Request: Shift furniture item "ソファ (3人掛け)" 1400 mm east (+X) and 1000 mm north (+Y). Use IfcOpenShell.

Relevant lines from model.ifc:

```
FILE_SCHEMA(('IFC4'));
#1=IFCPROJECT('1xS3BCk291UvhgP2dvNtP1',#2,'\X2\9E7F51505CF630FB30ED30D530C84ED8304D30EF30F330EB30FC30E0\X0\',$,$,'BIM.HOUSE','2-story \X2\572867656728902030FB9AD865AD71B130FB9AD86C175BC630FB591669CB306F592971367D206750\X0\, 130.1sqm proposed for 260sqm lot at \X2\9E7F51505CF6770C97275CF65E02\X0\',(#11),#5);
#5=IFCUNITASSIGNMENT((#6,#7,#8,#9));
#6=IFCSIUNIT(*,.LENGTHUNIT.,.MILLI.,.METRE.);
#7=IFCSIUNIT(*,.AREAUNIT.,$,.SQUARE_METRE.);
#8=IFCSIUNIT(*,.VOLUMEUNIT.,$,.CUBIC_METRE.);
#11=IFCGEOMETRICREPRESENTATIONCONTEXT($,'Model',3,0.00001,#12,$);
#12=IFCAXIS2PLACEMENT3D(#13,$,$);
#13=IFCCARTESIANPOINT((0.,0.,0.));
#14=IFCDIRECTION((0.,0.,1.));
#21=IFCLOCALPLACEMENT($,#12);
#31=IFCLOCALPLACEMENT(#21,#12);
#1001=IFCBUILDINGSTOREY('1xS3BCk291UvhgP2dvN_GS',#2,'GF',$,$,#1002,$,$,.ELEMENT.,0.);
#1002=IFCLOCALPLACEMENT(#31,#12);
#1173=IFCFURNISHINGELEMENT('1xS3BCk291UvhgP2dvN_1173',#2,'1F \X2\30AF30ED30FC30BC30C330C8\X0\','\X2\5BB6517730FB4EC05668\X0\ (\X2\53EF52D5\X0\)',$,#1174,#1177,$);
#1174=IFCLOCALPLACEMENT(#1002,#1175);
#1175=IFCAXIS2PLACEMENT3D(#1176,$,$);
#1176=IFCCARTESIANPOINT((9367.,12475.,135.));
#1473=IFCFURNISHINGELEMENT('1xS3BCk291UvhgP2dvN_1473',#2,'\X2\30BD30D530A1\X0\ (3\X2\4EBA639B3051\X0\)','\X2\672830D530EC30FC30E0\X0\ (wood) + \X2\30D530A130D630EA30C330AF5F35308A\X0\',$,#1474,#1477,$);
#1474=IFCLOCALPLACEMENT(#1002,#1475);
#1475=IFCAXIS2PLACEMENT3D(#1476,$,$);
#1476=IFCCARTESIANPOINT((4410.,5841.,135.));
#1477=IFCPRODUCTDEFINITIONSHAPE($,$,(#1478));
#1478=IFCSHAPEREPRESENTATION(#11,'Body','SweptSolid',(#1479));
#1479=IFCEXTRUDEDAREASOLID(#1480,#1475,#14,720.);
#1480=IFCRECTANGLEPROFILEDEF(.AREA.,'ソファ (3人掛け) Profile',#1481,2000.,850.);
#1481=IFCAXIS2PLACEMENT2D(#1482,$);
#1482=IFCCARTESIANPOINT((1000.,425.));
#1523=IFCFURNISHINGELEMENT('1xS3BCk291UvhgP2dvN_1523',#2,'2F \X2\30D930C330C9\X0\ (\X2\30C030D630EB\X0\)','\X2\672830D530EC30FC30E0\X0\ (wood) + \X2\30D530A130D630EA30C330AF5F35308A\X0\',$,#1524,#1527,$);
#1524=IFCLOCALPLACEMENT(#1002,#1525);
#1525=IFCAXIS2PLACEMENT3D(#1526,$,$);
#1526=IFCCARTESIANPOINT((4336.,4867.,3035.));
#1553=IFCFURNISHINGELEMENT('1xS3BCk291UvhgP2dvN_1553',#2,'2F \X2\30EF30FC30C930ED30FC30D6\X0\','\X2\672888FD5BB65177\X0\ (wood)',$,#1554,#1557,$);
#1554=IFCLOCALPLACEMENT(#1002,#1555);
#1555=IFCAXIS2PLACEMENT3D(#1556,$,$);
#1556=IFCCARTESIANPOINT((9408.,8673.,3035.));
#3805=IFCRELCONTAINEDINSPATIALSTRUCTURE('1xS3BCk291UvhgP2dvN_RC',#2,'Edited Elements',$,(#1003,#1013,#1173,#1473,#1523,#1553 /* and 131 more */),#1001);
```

```python
import ifcopenshell
import ifcopenshell.api.geometry
import ifcopenshell.util.placement

model = ifcopenshell.open("model.ifc")

item = model.by_id(1473)
matrix = ifcopenshell.util.placement.get_local_placement(item.ObjectPlacement)
matrix[0, 3] += 1400.0
matrix[1, 3] += 1000.0
ifcopenshell.api.geometry.edit_object_placement(model, product=item, matrix=matrix, is_si=False)

print(ifcopenshell.util.placement.get_local_placement(item.ObjectPlacement).round(3) + 0.0)

model.write("model_edited.ifc")
```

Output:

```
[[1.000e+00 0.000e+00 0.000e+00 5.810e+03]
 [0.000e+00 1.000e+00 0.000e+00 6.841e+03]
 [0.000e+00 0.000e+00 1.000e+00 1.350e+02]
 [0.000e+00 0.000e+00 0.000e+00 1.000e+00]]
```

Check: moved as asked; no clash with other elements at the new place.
